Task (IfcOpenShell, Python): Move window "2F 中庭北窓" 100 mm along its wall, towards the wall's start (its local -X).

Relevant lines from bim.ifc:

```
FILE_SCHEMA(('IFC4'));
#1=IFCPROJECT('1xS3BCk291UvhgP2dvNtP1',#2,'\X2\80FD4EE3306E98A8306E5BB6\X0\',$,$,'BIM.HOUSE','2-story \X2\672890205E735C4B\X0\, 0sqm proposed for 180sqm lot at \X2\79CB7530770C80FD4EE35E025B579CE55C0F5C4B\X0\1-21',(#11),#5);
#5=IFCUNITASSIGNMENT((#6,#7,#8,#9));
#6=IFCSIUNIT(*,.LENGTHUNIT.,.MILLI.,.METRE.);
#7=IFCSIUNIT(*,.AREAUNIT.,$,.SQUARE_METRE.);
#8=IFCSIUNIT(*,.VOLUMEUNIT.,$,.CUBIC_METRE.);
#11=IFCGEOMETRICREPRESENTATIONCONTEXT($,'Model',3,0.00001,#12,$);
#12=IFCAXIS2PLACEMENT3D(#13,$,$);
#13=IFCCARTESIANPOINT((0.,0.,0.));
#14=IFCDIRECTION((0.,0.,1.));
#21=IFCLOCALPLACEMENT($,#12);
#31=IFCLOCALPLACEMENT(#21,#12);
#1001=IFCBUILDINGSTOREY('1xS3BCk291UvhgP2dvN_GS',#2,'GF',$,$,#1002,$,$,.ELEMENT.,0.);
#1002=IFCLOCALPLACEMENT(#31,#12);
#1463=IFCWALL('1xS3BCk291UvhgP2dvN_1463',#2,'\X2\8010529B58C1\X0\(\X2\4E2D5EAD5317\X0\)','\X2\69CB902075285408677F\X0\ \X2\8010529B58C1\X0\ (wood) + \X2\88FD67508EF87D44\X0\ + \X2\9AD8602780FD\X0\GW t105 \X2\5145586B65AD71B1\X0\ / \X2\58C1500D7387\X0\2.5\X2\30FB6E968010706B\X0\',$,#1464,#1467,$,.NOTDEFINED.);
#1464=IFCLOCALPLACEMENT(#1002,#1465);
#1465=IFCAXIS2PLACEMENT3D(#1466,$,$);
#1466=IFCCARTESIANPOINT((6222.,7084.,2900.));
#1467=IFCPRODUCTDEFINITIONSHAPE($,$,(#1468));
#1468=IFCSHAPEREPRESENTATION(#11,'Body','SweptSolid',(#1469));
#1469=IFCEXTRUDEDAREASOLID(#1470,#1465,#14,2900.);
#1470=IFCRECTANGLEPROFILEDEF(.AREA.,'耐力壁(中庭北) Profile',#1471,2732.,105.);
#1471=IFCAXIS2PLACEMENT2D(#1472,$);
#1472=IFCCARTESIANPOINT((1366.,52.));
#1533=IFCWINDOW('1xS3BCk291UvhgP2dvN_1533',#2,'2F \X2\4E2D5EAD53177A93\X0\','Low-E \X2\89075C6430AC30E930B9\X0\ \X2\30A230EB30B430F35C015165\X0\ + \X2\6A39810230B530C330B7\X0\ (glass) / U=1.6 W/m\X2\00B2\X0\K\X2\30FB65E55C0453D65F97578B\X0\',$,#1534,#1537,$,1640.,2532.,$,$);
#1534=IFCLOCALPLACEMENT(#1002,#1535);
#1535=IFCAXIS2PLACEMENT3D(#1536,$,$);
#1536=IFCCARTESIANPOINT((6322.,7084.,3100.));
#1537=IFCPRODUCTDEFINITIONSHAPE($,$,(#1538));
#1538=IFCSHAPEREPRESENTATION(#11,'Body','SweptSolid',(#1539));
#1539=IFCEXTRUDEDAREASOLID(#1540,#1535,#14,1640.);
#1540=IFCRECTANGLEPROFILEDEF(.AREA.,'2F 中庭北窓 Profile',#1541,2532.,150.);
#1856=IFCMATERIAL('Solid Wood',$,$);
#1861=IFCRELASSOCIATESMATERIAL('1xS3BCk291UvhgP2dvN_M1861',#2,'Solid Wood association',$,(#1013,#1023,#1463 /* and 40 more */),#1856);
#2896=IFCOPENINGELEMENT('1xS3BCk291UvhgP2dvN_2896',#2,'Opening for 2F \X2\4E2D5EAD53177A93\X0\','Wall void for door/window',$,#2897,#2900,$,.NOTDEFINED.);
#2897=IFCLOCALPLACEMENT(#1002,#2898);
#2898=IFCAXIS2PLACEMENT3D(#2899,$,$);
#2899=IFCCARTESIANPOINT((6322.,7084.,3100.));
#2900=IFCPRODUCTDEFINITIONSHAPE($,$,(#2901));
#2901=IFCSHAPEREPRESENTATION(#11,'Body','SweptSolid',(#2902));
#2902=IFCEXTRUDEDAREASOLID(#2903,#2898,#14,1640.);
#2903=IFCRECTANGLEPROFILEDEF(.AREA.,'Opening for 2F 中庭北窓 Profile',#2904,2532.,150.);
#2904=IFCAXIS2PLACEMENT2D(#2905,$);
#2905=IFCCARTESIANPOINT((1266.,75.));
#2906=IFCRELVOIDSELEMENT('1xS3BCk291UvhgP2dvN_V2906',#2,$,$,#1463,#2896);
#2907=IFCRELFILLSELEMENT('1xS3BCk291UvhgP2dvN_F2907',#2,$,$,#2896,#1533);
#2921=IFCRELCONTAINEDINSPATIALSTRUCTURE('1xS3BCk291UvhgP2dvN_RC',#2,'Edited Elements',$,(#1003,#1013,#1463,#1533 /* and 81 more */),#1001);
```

```python
import ifcopenshell
import ifcopenshell.api.geometry
import ifcopenshell.util.placement
import ifcopenshell.util.unit

model = ifcopenshell.open("bim.ifc")
unit_scale = ifcopenshell.util.unit.calculate_unit_scale(model)

window = model.by_guid("1xS3BCk291UvhgP2dvN_1533")
opening = window.FillsVoids[0].RelatingOpeningElement
wall = opening.VoidsElements[0].RelatingBuildingElement

wall_matrix = ifcopenshell.util.placement.get_local_placement(wall.ObjectPlacement)
shift = wall_matrix[:3, 0] * -0.1 / unit_scale
before = ifcopenshell.util.placement.get_local_placement(window.ObjectPlacement)[:3, 3].copy()

# The window is not placed relative to its opening, so move both.
for product in (opening, window):
    matrix = ifcopenshell.util.placement.get_local_placement(product.ObjectPlacement)
    matrix[:3, 3] += shift
    ifcopenshell.api.geometry.edit_object_placement(model, product=product, matrix=matrix, is_si=False)

after = ifcopenshell.util.placement.get_local_placement(window.ObjectPlacement)[:3, 3]
print("window moved by", (after - before).round(3) + 0.0)

model.write("bim_rev.ifc")
```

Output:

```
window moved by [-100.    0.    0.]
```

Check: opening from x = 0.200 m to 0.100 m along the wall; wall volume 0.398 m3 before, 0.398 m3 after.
